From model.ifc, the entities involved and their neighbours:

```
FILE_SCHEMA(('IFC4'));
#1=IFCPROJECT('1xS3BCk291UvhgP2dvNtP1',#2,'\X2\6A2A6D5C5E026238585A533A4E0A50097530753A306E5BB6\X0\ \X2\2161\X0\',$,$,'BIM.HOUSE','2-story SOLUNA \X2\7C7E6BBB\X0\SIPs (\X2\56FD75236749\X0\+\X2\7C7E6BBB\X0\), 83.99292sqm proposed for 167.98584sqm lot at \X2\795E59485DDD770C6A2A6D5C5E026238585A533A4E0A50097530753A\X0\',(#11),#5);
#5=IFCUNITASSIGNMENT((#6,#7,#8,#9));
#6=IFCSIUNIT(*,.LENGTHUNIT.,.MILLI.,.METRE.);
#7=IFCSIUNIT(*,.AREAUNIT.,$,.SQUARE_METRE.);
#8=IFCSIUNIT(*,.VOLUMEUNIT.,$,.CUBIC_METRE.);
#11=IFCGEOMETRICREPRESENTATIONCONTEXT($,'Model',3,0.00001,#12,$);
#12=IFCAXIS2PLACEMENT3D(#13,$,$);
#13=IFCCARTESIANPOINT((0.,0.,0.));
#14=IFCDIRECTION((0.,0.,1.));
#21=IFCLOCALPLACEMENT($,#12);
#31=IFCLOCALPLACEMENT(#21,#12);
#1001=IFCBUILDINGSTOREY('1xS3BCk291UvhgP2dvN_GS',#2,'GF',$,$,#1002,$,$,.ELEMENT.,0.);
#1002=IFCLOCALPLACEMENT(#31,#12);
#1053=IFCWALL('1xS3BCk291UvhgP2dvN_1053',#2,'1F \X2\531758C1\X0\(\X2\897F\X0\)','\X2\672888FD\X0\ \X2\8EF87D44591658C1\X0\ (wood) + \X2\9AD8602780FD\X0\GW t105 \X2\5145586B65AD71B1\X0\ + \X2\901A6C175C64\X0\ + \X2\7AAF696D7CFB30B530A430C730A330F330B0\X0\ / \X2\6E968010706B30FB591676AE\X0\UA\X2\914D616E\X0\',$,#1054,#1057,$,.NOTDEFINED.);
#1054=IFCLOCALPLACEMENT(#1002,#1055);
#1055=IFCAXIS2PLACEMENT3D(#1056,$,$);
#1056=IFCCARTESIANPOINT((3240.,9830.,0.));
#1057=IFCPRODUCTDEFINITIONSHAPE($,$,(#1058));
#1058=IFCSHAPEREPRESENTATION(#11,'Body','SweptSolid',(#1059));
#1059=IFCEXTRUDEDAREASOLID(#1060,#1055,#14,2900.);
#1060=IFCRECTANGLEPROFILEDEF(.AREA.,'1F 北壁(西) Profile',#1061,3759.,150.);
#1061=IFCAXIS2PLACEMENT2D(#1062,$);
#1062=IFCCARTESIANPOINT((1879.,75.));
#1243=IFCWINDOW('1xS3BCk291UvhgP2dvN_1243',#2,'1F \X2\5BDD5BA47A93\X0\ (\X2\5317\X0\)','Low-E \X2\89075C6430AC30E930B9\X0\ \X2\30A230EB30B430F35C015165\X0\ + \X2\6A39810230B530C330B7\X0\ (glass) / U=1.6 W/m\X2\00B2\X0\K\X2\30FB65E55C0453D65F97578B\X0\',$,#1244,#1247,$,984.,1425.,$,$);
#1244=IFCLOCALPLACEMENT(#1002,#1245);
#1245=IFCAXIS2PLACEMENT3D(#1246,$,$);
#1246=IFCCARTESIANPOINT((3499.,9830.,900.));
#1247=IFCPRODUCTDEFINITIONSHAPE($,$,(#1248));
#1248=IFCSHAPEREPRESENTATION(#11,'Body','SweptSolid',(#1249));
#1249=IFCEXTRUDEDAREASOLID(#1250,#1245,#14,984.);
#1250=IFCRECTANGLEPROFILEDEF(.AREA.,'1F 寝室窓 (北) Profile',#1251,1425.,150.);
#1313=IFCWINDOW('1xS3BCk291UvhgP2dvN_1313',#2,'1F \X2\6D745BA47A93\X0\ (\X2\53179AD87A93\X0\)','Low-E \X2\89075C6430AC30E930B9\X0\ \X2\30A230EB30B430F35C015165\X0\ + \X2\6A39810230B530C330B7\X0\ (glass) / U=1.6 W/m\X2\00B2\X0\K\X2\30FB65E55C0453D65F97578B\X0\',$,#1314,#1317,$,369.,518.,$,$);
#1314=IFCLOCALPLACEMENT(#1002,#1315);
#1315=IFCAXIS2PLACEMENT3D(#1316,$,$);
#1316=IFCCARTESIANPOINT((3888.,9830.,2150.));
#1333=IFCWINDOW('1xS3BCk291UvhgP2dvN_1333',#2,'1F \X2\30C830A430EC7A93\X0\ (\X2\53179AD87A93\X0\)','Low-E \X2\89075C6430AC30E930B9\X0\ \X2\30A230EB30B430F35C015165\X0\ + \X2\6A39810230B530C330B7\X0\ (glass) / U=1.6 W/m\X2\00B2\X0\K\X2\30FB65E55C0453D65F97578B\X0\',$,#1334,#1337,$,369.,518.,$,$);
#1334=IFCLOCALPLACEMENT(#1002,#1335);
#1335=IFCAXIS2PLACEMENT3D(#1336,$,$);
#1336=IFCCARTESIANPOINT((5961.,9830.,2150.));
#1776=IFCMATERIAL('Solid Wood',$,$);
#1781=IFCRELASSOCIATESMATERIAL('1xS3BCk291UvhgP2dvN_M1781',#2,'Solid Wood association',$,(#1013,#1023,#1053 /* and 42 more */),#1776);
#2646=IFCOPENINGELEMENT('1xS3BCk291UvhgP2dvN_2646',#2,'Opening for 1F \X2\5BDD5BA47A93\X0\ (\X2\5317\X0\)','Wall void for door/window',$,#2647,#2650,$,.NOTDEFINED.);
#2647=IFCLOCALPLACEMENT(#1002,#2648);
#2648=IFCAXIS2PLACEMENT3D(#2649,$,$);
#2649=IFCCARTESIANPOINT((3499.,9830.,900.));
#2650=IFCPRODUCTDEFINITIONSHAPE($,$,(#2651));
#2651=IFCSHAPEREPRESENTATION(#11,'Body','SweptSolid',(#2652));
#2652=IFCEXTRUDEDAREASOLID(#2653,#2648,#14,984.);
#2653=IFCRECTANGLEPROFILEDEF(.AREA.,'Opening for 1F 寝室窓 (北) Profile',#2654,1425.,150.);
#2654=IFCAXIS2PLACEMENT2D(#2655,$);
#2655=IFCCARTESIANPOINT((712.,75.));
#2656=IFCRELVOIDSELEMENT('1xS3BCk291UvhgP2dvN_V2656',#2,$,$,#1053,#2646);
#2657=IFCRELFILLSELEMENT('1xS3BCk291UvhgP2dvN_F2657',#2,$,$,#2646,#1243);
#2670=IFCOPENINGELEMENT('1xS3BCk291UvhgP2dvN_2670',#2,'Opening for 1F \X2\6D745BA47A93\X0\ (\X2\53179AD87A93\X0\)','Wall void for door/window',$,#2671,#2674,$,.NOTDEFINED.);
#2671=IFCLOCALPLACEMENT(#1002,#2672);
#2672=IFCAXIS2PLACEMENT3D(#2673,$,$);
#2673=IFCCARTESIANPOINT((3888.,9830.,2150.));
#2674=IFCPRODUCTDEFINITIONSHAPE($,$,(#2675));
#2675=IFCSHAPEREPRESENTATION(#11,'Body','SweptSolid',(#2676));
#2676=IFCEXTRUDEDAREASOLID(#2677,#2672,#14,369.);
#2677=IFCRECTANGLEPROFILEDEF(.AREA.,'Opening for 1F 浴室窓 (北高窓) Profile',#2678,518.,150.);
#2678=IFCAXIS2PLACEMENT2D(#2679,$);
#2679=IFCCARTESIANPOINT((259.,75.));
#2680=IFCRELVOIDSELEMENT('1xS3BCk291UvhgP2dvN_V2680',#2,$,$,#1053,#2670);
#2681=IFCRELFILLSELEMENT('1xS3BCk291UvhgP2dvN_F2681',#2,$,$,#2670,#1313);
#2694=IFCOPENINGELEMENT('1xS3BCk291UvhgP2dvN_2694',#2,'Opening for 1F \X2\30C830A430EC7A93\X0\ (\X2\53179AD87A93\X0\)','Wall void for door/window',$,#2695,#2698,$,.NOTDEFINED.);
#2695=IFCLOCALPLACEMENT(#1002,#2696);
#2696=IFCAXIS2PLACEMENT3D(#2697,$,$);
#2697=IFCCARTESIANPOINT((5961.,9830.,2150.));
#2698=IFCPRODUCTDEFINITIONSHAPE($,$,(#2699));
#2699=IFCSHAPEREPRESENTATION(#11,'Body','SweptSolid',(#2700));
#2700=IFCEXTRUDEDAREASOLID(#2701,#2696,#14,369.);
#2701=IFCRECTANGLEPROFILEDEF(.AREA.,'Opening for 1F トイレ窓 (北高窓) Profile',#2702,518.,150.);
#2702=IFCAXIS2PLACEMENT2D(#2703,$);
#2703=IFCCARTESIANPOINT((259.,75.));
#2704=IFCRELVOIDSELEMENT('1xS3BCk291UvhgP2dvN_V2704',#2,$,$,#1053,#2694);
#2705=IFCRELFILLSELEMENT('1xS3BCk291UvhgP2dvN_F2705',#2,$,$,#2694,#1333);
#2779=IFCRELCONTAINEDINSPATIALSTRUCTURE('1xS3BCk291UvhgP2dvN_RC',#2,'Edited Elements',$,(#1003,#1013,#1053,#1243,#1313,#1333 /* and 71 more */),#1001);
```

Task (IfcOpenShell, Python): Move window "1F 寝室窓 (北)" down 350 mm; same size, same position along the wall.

```python
import numpy as np
import ifcopenshell
import ifcopenshell.api.geometry
import ifcopenshell.util.placement
import ifcopenshell.util.unit

model = ifcopenshell.open("model.ifc")
unit_scale = ifcopenshell.util.unit.calculate_unit_scale(model)

window = model.by_guid("1xS3BCk291UvhgP2dvN_1243")
opening = window.FillsVoids[0].RelatingOpeningElement
dz = -350.0

shift = np.array([0.0, 0.0, dz])
# The window is not placed relative to its opening, so move both.
for product in (opening, window):
    matrix = ifcopenshell.util.placement.get_local_placement(product.ObjectPlacement)
    matrix[:3, 3] += shift
    ifcopenshell.api.geometry.edit_object_placement(model, product=product, matrix=matrix, is_si=False)

print(f"moved by {dz * unit_scale:+.3f} m")

model.write("model_v2.ifc")
```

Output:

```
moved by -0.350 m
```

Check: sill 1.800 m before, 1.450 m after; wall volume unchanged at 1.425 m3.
